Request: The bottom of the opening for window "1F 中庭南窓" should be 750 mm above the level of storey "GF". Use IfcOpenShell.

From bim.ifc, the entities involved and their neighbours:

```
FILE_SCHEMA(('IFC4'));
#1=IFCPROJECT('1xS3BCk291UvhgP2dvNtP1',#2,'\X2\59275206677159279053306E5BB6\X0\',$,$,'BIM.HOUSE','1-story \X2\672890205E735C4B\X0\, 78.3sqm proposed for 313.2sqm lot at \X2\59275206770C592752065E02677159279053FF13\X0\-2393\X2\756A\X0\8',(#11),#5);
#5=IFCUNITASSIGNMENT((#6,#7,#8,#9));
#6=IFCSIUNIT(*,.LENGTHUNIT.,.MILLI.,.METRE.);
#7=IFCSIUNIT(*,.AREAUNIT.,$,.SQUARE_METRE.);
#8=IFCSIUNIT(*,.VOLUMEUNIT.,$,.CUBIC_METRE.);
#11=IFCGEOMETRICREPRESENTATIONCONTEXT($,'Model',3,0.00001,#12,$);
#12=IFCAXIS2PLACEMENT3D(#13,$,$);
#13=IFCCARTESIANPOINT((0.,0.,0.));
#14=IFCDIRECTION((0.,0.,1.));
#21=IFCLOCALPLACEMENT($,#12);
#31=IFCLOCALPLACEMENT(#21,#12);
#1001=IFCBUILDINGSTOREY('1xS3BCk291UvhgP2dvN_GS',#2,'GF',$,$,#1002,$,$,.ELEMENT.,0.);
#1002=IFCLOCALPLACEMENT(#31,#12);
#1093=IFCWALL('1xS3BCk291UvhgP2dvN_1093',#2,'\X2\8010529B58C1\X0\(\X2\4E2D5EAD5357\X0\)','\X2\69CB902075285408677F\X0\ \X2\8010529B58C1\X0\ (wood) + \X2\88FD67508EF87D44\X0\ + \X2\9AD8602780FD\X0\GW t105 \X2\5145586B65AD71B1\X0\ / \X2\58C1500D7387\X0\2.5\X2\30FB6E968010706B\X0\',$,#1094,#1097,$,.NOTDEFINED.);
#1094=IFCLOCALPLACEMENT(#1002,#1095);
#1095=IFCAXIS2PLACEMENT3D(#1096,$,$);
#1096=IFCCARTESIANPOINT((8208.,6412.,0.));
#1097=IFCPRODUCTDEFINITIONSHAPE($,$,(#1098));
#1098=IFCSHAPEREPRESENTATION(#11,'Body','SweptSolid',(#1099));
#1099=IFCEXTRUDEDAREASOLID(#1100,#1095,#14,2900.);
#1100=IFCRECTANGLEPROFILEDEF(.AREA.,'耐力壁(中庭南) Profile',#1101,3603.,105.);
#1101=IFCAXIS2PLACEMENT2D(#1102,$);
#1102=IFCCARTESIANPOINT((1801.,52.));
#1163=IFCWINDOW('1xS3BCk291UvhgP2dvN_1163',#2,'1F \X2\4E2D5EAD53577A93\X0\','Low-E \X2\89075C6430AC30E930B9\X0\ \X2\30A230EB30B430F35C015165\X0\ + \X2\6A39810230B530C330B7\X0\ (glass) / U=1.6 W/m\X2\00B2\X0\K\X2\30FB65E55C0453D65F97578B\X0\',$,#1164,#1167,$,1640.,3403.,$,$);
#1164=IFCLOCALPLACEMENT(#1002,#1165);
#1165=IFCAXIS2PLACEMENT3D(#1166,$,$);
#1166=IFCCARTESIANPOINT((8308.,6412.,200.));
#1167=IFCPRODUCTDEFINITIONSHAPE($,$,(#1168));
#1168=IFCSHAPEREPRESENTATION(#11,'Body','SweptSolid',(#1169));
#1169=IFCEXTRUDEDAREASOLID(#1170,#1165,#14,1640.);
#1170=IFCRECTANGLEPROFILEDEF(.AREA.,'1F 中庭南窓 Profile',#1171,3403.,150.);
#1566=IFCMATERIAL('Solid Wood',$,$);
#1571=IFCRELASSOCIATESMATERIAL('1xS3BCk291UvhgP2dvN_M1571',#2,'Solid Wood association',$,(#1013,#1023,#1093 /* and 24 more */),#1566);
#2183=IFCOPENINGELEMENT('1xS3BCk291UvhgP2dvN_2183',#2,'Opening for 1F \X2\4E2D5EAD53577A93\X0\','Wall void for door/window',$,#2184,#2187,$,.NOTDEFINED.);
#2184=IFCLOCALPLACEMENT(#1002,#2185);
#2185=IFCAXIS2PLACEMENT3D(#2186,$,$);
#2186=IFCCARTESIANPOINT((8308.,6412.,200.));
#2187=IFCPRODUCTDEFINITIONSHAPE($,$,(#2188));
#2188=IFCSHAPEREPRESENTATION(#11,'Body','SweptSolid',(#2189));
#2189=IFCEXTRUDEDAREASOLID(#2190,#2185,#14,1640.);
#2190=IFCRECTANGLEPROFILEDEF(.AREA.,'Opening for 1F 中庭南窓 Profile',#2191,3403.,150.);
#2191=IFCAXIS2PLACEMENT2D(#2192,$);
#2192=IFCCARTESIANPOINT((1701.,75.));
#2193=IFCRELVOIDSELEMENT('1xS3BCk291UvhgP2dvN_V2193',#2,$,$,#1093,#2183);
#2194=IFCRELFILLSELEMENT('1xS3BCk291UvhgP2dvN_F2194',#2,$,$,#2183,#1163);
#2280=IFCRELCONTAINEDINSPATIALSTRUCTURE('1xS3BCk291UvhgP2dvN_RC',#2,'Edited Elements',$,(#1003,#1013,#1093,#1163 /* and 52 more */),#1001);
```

```python
import numpy as np
import ifcopenshell
import ifcopenshell.api.geometry
import ifcopenshell.geom
import ifcopenshell.util.element
import ifcopenshell.util.placement
import ifcopenshell.util.shape
import ifcopenshell.util.unit

model = ifcopenshell.open("bim.ifc")
unit_scale = ifcopenshell.util.unit.calculate_unit_scale(model)

window = model.by_guid("1xS3BCk291UvhgP2dvN_1163")
opening = window.FillsVoids[0].RelatingOpeningElement
storey = ifcopenshell.util.element.get_container(window, ifc_class="IfcBuildingStorey")
level = ifcopenshell.util.placement.get_local_placement(storey.ObjectPlacement)[2, 3]

# The opening's origin need not be at the sill, so measure its lowest point.
shape = ifcopenshell.geom.create_shape(ifcopenshell.geom.settings(), opening)
bottom = ifcopenshell.util.shape.get_shape_bottom_elevation(shape, shape.geometry) / unit_scale
dz = level + 0.75 / unit_scale - bottom

shift = np.array([0.0, 0.0, dz])
# The window is not placed relative to its opening, so move both.
for product in (opening, window):
    matrix = ifcopenshell.util.placement.get_local_placement(product.ObjectPlacement)
    matrix[:3, 3] += shift
    ifcopenshell.api.geometry.edit_object_placement(model, product=product, matrix=matrix, is_si=False)

print(f"moved by {dz * unit_scale:+.3f} m")

model.write("bim-out.ifc")
```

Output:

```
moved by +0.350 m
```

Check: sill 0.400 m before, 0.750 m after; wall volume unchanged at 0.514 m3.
